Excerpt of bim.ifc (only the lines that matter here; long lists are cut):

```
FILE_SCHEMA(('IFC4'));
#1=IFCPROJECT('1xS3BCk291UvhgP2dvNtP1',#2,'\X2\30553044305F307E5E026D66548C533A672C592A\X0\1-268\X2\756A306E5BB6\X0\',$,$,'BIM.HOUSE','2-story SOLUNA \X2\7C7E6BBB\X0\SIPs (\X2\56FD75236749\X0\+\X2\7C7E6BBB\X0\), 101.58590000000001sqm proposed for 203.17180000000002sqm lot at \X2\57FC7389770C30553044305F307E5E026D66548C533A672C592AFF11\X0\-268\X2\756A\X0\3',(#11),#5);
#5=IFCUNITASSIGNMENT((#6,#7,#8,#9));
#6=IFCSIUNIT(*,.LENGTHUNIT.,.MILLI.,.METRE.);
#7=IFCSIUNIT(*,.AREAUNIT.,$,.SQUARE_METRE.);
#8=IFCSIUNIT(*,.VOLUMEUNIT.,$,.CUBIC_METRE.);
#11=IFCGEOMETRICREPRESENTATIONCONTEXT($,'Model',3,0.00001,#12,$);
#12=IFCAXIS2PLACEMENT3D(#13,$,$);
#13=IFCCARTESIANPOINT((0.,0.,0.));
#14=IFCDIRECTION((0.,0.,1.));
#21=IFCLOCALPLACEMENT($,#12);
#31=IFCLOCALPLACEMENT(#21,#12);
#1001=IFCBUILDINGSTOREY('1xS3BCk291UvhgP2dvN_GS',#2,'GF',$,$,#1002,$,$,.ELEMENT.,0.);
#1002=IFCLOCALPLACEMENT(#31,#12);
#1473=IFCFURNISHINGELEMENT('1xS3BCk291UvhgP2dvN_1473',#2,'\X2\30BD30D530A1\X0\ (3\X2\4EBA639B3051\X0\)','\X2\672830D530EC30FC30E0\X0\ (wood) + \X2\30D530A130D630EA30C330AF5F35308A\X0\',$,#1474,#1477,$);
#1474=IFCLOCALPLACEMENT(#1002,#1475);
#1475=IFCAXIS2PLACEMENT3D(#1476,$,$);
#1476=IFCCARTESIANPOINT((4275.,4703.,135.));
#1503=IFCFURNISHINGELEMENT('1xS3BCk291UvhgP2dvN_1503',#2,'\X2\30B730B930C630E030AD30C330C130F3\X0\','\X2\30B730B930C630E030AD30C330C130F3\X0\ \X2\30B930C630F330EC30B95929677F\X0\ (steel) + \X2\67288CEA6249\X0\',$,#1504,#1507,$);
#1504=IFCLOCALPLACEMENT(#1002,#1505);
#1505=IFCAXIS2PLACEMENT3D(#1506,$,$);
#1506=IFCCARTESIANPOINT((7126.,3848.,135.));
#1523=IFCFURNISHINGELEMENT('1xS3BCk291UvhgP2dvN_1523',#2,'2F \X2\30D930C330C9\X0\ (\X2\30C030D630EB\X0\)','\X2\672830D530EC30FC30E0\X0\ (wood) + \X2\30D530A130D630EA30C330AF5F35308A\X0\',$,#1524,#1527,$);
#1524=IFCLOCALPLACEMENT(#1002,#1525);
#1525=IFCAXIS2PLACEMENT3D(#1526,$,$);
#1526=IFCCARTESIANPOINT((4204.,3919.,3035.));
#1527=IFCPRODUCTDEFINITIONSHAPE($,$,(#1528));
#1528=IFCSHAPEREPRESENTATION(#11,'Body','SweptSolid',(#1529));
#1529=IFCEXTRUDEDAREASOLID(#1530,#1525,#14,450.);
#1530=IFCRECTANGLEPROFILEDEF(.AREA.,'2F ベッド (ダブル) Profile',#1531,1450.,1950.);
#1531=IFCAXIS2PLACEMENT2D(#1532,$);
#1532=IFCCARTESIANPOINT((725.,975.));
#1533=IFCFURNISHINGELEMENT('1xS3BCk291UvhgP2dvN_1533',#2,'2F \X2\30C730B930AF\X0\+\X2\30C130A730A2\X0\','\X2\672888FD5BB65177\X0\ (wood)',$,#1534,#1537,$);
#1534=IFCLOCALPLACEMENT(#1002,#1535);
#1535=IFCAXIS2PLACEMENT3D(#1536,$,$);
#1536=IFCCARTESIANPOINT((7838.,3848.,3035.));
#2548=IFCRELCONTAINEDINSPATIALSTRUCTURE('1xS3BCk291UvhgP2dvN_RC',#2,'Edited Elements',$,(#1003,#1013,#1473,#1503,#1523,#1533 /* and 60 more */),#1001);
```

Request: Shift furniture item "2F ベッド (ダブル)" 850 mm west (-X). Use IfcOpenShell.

```python
import ifcopenshell
import ifcopenshell.api.geometry
import ifcopenshell.util.placement
import ifcopenshell.util.unit

model = ifcopenshell.open("bim.ifc")
unit_scale = ifcopenshell.util.unit.calculate_unit_scale(model)

item = model.by_guid("1xS3BCk291UvhgP2dvN_1523")
matrix = ifcopenshell.util.placement.get_local_placement(item.ObjectPlacement)
matrix[0, 3] -= 0.85 / unit_scale
ifcopenshell.api.geometry.edit_object_placement(model, product=item, matrix=matrix, is_si=False)

print(ifcopenshell.util.placement.get_local_placement(item.ObjectPlacement).round(3) + 0.0)

model.write("bim_rev.ifc")
```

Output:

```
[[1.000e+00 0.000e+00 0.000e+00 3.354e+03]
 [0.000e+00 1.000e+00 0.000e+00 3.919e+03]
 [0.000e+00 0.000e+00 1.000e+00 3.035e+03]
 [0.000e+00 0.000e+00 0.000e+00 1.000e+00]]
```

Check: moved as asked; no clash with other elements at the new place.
